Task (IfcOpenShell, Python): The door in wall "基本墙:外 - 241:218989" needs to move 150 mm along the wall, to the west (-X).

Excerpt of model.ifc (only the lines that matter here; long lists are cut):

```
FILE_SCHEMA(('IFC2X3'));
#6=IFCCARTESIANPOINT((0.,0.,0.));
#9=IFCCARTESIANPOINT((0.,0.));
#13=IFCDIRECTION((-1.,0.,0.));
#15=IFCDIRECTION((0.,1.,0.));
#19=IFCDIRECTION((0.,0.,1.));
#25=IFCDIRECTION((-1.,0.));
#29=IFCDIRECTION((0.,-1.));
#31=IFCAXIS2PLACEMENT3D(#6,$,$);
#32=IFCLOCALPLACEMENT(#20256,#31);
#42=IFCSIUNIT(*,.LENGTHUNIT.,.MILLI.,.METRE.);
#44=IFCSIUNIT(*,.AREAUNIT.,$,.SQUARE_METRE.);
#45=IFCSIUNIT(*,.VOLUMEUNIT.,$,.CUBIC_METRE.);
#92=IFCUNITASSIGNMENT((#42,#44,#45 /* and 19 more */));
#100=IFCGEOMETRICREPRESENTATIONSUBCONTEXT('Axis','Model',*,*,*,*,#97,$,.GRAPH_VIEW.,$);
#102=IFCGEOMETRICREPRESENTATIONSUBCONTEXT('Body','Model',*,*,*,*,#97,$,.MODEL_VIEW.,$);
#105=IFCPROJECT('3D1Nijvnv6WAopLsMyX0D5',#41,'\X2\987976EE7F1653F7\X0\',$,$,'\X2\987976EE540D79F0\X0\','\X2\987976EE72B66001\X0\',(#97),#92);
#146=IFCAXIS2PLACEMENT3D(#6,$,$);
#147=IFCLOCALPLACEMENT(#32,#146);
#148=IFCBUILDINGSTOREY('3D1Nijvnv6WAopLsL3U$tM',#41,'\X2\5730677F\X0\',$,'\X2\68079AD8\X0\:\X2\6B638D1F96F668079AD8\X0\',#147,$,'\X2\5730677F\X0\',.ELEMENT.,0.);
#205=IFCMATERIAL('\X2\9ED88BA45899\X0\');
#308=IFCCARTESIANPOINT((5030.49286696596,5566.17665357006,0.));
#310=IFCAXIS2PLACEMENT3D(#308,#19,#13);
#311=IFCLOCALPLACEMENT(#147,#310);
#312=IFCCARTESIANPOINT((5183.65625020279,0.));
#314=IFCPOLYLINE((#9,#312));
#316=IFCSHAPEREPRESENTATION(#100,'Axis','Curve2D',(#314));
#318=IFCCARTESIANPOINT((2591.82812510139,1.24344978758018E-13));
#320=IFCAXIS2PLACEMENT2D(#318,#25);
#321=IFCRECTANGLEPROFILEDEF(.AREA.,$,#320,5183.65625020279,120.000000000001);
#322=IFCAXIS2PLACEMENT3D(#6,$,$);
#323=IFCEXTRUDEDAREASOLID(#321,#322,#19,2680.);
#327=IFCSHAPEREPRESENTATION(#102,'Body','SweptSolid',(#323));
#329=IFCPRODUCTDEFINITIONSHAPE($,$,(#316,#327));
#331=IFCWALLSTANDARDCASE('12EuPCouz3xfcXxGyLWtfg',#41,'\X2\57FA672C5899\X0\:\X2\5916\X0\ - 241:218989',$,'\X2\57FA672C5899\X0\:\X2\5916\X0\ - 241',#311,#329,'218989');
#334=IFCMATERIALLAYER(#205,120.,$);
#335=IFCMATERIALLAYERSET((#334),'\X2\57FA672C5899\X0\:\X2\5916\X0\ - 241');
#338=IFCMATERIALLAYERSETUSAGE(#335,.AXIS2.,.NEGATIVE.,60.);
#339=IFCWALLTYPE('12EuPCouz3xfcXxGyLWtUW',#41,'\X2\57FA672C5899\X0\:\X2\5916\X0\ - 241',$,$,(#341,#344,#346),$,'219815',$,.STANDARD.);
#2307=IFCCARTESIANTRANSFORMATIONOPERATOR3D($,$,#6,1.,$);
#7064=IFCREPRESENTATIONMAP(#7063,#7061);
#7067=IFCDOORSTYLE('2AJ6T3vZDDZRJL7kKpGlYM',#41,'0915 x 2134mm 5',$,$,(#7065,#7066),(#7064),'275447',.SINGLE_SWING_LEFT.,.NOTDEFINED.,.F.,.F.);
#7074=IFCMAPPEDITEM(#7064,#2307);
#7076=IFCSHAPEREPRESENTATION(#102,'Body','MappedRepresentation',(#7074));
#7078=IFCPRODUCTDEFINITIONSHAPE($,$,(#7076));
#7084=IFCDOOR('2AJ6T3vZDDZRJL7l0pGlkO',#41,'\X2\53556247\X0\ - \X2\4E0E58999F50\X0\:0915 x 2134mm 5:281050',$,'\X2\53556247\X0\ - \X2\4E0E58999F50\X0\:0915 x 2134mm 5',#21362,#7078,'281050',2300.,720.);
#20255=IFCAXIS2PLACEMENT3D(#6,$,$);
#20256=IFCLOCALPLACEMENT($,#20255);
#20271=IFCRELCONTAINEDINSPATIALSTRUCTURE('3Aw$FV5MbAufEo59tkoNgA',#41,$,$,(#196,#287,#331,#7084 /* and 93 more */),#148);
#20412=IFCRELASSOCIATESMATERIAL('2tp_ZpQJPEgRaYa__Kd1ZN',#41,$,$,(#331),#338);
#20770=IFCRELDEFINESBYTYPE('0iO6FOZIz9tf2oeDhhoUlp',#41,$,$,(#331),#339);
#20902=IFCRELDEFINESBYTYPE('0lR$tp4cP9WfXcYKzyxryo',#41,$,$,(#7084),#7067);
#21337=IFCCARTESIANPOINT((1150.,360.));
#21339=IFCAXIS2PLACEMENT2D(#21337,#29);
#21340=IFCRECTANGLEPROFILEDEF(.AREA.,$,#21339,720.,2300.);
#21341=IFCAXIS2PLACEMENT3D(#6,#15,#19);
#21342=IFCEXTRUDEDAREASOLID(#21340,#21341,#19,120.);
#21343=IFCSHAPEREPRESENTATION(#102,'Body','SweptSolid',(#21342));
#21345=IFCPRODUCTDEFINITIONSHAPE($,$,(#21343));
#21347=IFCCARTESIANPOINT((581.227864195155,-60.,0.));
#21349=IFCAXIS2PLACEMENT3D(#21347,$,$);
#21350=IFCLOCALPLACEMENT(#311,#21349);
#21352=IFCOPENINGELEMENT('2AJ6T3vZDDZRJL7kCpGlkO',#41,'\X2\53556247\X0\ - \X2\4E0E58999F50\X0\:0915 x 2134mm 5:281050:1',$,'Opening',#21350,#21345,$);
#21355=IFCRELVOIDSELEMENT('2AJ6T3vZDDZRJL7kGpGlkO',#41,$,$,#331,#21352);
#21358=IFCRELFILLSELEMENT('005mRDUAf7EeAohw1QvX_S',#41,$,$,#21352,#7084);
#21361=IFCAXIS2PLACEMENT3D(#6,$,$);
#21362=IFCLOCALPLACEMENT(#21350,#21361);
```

```python
import ifcopenshell
import ifcopenshell.api.geometry
import ifcopenshell.util.placement
import ifcopenshell.util.unit

model = ifcopenshell.open("model.ifc")
unit_scale = ifcopenshell.util.unit.calculate_unit_scale(model)

door = model.by_id(7084)
opening = door.FillsVoids[0].RelatingOpeningElement
wall = opening.VoidsElements[0].RelatingBuildingElement

wall_matrix = ifcopenshell.util.placement.get_local_placement(wall.ObjectPlacement)
shift = wall_matrix[:3, 0] * 0.15 / unit_scale
before = ifcopenshell.util.placement.get_local_placement(door.ObjectPlacement)[:3, 3].copy()

# The door is placed relative to its opening, so it follows when the opening moves.
matrix = ifcopenshell.util.placement.get_local_placement(opening.ObjectPlacement)
matrix[:3, 3] += shift
ifcopenshell.api.geometry.edit_object_placement(
    model, product=opening, matrix=matrix, is_si=False, should_transform_children=True
)

after = ifcopenshell.util.placement.get_local_placement(door.ObjectPlacement)[:3, 3]
print("door moved by", (after - before).round(3) + 0.0)

model.write("model_edited.ifc")
```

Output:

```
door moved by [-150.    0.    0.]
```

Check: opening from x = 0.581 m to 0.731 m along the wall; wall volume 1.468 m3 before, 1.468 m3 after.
